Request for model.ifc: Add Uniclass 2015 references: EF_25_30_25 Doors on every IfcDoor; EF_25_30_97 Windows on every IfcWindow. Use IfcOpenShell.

First a look at what the model holds.

```python
import ifcopenshell

model = ifcopenshell.open("model.ifc")
print(model.schema)
print("classifications:", [c.Name for c in model.by_type("IfcClassification")])
for ifc_class in ("IfcDoor", "IfcRoof", "IfcStair", "IfcWall", "IfcWindow"):
    print(ifc_class, len(model.by_type(ifc_class)))
```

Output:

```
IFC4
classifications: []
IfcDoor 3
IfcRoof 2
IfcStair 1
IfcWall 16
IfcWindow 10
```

```python
import ifcopenshell
import ifcopenshell.api.classification

model = ifcopenshell.open("model.ifc")

system = ifcopenshell.api.classification.add_classification(model, classification="Uniclass 2015")

codes = {
    "IfcDoor": ("EF_25_30_25", "Doors"),
    "IfcWindow": ("EF_25_30_97", "Windows"),
}
for ifc_class, (code, name) in codes.items():
    products = model.by_type(ifc_class)
    ifcopenshell.api.classification.add_reference(
        model, products=products, classification=system, identification=code, name=name
    )
    print(code, len(products))

model.write("model_edited.ifc")
```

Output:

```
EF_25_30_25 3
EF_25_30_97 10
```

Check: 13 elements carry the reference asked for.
